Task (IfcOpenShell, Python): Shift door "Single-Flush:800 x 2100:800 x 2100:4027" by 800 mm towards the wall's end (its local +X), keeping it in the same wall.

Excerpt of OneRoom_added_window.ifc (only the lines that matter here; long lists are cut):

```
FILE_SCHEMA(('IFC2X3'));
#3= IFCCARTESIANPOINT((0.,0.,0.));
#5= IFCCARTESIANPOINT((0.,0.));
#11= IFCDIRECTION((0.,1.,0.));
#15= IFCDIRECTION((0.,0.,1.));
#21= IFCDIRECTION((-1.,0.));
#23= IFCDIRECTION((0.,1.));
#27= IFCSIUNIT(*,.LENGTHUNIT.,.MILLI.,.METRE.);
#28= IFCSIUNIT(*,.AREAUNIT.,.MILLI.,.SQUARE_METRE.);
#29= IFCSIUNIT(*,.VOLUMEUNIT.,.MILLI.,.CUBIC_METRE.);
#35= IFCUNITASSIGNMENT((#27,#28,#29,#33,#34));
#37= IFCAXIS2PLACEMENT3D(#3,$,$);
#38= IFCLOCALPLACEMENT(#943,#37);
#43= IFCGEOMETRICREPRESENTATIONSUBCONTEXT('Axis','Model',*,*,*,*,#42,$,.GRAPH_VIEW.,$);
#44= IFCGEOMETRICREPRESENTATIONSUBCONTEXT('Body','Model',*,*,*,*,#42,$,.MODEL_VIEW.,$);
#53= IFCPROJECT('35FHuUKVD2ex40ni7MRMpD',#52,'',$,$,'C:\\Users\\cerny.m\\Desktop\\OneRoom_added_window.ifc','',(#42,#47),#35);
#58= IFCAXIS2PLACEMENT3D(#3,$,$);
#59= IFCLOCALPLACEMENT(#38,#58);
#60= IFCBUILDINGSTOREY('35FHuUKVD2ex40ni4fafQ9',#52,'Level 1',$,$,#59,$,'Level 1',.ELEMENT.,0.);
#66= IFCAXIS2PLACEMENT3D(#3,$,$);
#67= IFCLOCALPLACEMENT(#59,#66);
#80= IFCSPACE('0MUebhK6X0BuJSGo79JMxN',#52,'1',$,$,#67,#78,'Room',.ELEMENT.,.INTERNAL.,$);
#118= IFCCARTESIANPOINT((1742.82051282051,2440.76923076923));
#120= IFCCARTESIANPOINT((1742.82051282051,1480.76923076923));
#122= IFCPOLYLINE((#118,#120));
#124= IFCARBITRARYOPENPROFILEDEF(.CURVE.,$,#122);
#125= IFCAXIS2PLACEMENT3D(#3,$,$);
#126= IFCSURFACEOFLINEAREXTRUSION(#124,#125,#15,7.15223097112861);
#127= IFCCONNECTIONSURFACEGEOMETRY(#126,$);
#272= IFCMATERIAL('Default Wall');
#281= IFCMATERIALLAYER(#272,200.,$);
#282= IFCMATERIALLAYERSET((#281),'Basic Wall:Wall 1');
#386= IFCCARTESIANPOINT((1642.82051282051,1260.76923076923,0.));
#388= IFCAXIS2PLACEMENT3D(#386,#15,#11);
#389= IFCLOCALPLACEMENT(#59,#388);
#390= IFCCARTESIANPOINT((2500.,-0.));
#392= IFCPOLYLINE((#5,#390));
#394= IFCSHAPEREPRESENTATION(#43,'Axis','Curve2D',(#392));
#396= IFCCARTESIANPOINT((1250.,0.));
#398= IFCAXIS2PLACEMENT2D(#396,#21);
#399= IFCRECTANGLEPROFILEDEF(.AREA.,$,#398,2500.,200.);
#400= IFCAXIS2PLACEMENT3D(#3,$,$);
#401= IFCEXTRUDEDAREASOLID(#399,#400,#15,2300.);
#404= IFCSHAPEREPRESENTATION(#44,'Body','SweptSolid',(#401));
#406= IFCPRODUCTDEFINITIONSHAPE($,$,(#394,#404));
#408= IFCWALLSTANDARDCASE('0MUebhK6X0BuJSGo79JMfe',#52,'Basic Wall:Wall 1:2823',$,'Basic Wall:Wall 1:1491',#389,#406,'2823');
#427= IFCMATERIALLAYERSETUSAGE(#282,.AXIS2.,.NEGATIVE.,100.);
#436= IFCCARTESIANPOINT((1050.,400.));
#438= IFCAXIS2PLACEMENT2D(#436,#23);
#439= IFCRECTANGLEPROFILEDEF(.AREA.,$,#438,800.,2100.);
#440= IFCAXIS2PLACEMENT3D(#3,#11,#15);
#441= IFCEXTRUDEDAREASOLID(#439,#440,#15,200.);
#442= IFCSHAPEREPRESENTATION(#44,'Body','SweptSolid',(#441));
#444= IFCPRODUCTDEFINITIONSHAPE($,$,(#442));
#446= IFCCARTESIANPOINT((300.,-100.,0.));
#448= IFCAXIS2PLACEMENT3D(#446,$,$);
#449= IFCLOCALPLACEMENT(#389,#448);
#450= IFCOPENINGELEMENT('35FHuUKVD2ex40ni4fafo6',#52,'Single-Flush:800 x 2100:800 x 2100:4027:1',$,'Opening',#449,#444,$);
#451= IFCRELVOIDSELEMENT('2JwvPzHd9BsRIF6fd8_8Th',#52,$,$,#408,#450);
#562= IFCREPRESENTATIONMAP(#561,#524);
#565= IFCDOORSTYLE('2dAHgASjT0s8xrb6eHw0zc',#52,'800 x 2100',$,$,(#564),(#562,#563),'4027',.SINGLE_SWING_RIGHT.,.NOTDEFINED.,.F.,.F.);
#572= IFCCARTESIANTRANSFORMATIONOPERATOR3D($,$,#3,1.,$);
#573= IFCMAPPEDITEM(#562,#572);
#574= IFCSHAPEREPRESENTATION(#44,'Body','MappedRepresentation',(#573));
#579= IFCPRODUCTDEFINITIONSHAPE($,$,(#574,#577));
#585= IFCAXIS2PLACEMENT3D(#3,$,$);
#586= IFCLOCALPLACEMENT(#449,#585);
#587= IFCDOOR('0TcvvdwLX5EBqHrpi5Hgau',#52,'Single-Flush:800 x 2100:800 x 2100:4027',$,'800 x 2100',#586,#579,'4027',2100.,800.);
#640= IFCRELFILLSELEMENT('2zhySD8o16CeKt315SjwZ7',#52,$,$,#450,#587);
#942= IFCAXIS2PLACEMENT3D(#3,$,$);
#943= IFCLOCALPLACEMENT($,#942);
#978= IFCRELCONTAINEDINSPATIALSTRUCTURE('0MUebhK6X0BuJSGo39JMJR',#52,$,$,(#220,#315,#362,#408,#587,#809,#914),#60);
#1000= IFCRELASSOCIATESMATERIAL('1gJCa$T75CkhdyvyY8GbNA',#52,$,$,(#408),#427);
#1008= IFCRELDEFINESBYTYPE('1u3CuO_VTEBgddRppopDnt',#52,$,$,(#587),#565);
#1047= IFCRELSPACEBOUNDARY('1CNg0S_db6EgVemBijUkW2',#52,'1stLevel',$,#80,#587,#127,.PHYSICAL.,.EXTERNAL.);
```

```python
import numpy as np
import ifcopenshell
import ifcopenshell.api.geometry
import ifcopenshell.util.placement
import ifcopenshell.util.unit

model = ifcopenshell.open("OneRoom_added_window.ifc")
unit_scale = ifcopenshell.util.unit.calculate_unit_scale(model)

door = model.by_guid("0TcvvdwLX5EBqHrpi5Hgau")
opening = door.FillsVoids[0].RelatingOpeningElement
wall = opening.VoidsElements[0].RelatingBuildingElement

wall_matrix = ifcopenshell.util.placement.get_local_placement(wall.ObjectPlacement)
shift = wall_matrix[:3, 0] * 0.8 / unit_scale
before = ifcopenshell.util.placement.get_local_placement(door.ObjectPlacement)[:3, 3].copy()

# The door is placed relative to its opening, so it follows when the opening moves.
matrix = ifcopenshell.util.placement.get_local_placement(opening.ObjectPlacement)
matrix[:3, 3] += shift
ifcopenshell.api.geometry.edit_object_placement(
    model, product=opening, matrix=matrix, is_si=False, should_transform_children=True
)

# Space boundary surfaces are stored in each space's coordinates; move them too.
for rel in door.ProvidesBoundaries:
    if not rel.ConnectionGeometry:
        continue
    surface = rel.ConnectionGeometry.SurfaceOnRelatingElement
    space_matrix = ifcopenshell.util.placement.get_local_placement(rel.RelatingSpace.ObjectPlacement)
    point = np.array(surface.Position.Location.Coordinates) + space_matrix[:3, :3].T @ shift
    surface.Position = model.createIfcAxis2Placement3D(
        model.createIfcCartesianPoint(point.tolist()), surface.Position.Axis, surface.Position.RefDirection
    )

after = ifcopenshell.util.placement.get_local_placement(door.ObjectPlacement)[:3, 3]
print("door moved by", (after - before).round(3) + 0.0)

model.write("OneRoom_added_window_rev.ifc")
```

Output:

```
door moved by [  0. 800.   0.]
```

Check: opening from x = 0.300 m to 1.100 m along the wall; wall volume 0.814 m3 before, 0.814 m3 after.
